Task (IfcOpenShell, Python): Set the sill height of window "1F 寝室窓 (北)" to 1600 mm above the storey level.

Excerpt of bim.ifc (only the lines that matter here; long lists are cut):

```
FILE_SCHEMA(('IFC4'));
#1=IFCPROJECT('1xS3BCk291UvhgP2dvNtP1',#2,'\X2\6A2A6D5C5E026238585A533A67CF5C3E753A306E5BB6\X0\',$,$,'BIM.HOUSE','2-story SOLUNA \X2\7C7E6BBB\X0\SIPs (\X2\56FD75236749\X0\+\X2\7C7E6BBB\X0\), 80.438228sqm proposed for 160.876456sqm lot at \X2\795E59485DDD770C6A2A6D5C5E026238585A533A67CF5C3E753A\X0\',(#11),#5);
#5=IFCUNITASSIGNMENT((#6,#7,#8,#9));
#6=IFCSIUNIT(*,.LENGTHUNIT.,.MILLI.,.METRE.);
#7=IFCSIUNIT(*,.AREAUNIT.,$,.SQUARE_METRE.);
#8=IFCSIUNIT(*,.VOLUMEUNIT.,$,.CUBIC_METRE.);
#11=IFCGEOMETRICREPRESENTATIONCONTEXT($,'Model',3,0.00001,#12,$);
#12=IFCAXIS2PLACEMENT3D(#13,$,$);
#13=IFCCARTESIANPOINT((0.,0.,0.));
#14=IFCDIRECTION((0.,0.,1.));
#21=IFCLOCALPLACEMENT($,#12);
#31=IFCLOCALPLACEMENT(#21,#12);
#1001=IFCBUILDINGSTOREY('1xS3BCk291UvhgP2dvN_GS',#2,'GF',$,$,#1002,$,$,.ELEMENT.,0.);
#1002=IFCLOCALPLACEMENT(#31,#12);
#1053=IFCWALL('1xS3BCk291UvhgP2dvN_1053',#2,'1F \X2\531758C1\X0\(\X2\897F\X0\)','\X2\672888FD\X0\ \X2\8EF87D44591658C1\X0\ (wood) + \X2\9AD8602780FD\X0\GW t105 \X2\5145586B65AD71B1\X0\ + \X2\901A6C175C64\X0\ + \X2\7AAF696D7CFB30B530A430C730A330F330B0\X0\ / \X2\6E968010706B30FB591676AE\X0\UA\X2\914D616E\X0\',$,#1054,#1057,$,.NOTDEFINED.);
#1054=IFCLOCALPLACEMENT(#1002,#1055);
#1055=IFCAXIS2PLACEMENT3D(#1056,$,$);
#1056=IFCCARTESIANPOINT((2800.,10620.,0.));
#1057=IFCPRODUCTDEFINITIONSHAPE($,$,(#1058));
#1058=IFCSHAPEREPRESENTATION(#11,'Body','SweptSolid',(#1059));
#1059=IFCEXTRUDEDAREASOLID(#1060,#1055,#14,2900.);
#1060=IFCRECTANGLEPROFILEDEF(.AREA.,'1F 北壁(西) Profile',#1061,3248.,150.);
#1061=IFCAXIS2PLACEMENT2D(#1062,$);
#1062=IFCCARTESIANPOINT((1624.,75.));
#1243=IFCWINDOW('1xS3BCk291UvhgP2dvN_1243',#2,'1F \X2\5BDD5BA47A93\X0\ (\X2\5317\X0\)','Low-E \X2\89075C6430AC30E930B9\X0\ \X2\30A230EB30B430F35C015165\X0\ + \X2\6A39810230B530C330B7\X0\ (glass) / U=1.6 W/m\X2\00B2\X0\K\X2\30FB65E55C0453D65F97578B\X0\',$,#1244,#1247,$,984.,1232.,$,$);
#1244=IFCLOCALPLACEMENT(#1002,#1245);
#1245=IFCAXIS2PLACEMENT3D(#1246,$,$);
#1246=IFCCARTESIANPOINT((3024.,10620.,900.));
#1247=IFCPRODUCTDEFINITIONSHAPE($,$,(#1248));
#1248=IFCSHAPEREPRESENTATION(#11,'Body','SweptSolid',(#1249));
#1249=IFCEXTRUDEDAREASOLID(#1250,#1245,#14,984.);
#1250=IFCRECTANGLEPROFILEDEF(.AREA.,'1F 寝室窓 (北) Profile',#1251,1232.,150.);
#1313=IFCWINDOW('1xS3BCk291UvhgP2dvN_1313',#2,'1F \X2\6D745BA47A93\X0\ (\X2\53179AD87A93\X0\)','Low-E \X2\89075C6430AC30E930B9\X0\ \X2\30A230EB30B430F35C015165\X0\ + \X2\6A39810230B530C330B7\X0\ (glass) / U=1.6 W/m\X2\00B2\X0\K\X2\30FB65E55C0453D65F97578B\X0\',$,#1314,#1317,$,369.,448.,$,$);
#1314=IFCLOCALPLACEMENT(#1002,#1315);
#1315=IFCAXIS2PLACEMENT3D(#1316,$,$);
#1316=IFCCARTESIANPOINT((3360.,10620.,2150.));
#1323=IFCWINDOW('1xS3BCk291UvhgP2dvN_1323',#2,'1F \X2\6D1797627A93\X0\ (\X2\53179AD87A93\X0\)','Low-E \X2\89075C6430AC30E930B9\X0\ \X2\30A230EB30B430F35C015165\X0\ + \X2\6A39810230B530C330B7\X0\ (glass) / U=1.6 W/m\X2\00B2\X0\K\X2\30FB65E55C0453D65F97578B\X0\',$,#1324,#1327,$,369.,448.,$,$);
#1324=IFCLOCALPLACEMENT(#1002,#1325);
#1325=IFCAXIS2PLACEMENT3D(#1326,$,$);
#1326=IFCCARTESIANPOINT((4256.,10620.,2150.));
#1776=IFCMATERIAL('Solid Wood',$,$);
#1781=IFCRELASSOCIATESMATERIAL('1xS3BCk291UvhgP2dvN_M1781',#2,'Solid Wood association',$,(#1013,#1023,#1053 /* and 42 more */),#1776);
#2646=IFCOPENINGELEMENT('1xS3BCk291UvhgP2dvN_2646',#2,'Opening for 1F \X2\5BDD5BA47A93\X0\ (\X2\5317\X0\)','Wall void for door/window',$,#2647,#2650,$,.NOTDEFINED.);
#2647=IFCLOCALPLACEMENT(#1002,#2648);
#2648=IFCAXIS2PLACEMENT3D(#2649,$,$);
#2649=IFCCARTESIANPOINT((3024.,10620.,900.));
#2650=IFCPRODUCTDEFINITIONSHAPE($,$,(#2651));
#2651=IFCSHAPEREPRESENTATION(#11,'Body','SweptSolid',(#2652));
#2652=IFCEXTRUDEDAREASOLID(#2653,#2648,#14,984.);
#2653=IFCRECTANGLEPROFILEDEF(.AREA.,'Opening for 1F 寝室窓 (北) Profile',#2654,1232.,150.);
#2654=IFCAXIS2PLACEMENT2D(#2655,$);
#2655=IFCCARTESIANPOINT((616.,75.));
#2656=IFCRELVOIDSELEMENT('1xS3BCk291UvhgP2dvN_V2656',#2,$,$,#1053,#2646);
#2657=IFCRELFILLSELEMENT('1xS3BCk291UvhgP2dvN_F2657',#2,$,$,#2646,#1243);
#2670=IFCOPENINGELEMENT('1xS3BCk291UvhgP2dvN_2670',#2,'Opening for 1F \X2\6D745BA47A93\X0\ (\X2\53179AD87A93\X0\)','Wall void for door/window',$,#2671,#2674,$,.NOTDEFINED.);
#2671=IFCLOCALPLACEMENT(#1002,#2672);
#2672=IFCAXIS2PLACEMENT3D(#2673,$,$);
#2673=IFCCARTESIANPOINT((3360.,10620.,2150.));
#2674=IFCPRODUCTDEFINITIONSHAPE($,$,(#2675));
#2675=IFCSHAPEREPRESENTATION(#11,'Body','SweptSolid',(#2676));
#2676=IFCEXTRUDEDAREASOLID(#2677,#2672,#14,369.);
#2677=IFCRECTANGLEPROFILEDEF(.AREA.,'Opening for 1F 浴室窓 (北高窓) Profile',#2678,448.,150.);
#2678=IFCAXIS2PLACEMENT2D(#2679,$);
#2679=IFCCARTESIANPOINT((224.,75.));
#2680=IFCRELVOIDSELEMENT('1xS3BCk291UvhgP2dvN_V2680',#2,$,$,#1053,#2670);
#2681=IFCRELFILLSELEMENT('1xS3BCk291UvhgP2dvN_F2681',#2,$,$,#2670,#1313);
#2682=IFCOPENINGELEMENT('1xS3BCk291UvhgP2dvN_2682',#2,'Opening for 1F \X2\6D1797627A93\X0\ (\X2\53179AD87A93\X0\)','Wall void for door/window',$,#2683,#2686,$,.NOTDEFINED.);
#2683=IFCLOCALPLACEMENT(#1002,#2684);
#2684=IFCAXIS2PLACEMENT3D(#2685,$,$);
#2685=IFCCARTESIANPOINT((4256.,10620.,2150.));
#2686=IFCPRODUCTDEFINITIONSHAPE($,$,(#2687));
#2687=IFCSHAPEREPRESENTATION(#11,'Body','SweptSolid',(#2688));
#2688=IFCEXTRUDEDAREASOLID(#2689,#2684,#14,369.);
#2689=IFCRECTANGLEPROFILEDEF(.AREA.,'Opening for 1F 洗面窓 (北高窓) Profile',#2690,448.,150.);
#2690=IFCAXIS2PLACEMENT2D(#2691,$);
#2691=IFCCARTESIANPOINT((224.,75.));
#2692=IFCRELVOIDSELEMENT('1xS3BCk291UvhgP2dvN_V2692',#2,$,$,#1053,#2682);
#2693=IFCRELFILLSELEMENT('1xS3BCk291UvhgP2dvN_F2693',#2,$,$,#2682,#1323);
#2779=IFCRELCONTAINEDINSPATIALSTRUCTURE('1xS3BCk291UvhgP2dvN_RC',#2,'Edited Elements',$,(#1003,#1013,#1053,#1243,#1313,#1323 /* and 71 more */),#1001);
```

```python
import numpy as np
import ifcopenshell
import ifcopenshell.api.geometry
import ifcopenshell.geom
import ifcopenshell.util.element
import ifcopenshell.util.placement
import ifcopenshell.util.shape
import ifcopenshell.util.unit

model = ifcopenshell.open("bim.ifc")
unit_scale = ifcopenshell.util.unit.calculate_unit_scale(model)

window = model.by_id(1243)
opening = window.FillsVoids[0].RelatingOpeningElement
storey = ifcopenshell.util.element.get_container(window, ifc_class="IfcBuildingStorey")
level = ifcopenshell.util.placement.get_local_placement(storey.ObjectPlacement)[2, 3]

# The opening's origin need not be at the sill, so measure its lowest point.
shape = ifcopenshell.geom.create_shape(ifcopenshell.geom.settings(), opening)
bottom = ifcopenshell.util.shape.get_shape_bottom_elevation(shape, shape.geometry) / unit_scale
dz = level + 1600.0 - bottom

shift = np.array([0.0, 0.0, dz])
# The window is not placed relative to its opening, so move both.
for product in (opening, window):
    matrix = ifcopenshell.util.placement.get_local_placement(product.ObjectPlacement)
    matrix[:3, 3] += shift
    ifcopenshell.api.geometry.edit_object_placement(model, product=product, matrix=matrix, is_si=False)

print(f"moved by {dz * unit_scale:+.3f} m")

model.write("bim_updated.ifc")
```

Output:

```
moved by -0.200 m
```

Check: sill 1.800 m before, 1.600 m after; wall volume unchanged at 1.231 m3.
